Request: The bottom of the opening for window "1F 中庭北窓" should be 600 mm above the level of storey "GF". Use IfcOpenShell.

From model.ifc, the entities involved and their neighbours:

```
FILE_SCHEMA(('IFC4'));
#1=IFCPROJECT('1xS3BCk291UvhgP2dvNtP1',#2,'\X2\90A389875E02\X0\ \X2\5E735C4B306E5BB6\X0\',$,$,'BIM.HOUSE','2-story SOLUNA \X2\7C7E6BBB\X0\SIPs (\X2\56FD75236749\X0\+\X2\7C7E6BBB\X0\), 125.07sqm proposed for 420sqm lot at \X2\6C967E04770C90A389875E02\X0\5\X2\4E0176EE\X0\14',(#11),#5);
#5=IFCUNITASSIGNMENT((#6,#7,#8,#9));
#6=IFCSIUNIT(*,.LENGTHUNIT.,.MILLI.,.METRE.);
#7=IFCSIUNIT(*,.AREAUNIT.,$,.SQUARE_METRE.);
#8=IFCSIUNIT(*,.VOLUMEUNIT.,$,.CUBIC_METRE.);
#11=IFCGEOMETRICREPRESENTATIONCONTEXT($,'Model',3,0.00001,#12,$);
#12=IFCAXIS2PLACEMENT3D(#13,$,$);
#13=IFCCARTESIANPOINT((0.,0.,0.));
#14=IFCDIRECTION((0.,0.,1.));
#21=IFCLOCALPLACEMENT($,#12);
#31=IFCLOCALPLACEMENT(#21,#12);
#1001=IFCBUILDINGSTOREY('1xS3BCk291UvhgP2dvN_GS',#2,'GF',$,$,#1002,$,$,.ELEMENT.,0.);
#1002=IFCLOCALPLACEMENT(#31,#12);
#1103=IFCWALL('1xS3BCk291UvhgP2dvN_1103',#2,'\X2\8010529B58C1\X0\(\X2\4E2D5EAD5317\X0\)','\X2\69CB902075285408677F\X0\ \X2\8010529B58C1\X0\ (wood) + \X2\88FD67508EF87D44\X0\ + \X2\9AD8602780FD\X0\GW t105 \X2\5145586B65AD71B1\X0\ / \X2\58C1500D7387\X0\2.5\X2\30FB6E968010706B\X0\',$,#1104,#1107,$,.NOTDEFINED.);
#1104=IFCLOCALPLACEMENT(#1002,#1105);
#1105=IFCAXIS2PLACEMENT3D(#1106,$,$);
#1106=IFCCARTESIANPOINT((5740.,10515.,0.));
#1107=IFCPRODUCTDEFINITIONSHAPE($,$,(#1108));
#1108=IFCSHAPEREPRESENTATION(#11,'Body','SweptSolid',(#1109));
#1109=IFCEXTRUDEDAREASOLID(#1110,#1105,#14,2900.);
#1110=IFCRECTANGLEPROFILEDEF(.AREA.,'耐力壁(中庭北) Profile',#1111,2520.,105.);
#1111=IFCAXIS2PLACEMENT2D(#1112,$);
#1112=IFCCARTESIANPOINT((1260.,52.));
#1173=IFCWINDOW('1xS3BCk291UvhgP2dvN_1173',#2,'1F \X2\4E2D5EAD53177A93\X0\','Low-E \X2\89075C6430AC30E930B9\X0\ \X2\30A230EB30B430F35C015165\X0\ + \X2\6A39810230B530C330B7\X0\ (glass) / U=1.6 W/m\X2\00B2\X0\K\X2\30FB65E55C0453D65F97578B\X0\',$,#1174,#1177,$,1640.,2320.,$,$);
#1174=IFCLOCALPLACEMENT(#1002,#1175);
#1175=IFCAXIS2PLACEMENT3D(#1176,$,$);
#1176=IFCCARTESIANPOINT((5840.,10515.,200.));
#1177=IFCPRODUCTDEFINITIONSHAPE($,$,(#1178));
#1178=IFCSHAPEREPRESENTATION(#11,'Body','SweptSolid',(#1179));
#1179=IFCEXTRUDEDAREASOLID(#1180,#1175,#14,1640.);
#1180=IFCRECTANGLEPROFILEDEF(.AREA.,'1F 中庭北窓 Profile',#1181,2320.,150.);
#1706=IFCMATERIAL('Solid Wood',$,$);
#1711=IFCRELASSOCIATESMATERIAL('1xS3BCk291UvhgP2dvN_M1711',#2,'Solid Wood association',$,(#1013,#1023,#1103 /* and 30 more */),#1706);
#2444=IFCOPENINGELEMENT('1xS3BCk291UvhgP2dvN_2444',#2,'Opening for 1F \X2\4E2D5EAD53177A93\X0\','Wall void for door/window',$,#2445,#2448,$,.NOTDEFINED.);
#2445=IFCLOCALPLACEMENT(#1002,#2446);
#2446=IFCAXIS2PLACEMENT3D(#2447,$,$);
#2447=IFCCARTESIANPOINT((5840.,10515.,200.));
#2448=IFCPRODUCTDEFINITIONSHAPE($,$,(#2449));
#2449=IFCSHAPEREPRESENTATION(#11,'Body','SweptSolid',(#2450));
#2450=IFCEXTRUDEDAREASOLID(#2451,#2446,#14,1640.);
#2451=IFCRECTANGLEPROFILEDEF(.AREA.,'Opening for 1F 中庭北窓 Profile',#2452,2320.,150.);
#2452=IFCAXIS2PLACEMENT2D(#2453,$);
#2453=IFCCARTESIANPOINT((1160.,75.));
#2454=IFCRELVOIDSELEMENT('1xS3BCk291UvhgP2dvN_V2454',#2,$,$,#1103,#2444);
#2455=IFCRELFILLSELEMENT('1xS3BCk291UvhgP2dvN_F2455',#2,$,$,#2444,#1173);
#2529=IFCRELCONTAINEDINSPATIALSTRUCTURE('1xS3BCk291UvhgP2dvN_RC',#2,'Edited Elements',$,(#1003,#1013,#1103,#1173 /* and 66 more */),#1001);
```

```python
import numpy as np
import ifcopenshell
import ifcopenshell.api.geometry
import ifcopenshell.geom
import ifcopenshell.util.element
import ifcopenshell.util.placement
import ifcopenshell.util.shape
import ifcopenshell.util.unit

model = ifcopenshell.open("model.ifc")
unit_scale = ifcopenshell.util.unit.calculate_unit_scale(model)

window = model.by_guid("1xS3BCk291UvhgP2dvN_1173")
opening = window.FillsVoids[0].RelatingOpeningElement
storey = ifcopenshell.util.element.get_container(window, ifc_class="IfcBuildingStorey")
level = ifcopenshell.util.placement.get_local_placement(storey.ObjectPlacement)[2, 3]

# The opening's origin need not be at the sill, so measure its lowest point.
shape = ifcopenshell.geom.create_shape(ifcopenshell.geom.settings(), opening)
bottom = ifcopenshell.util.shape.get_shape_bottom_elevation(shape, shape.geometry) / unit_scale
dz = level + 0.6 / unit_scale - bottom

shift = np.array([0.0, 0.0, dz])
# The window is not placed relative to its opening, so move both.
for product in (opening, window):
    matrix = ifcopenshell.util.placement.get_local_placement(product.ObjectPlacement)
    matrix[:3, 3] += shift
    ifcopenshell.api.geometry.edit_object_placement(model, product=product, matrix=matrix, is_si=False)

print(f"moved by {dz * unit_scale:+.3f} m")

model.write("model-out.ifc")
```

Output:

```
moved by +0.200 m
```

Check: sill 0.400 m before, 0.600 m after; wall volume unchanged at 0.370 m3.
